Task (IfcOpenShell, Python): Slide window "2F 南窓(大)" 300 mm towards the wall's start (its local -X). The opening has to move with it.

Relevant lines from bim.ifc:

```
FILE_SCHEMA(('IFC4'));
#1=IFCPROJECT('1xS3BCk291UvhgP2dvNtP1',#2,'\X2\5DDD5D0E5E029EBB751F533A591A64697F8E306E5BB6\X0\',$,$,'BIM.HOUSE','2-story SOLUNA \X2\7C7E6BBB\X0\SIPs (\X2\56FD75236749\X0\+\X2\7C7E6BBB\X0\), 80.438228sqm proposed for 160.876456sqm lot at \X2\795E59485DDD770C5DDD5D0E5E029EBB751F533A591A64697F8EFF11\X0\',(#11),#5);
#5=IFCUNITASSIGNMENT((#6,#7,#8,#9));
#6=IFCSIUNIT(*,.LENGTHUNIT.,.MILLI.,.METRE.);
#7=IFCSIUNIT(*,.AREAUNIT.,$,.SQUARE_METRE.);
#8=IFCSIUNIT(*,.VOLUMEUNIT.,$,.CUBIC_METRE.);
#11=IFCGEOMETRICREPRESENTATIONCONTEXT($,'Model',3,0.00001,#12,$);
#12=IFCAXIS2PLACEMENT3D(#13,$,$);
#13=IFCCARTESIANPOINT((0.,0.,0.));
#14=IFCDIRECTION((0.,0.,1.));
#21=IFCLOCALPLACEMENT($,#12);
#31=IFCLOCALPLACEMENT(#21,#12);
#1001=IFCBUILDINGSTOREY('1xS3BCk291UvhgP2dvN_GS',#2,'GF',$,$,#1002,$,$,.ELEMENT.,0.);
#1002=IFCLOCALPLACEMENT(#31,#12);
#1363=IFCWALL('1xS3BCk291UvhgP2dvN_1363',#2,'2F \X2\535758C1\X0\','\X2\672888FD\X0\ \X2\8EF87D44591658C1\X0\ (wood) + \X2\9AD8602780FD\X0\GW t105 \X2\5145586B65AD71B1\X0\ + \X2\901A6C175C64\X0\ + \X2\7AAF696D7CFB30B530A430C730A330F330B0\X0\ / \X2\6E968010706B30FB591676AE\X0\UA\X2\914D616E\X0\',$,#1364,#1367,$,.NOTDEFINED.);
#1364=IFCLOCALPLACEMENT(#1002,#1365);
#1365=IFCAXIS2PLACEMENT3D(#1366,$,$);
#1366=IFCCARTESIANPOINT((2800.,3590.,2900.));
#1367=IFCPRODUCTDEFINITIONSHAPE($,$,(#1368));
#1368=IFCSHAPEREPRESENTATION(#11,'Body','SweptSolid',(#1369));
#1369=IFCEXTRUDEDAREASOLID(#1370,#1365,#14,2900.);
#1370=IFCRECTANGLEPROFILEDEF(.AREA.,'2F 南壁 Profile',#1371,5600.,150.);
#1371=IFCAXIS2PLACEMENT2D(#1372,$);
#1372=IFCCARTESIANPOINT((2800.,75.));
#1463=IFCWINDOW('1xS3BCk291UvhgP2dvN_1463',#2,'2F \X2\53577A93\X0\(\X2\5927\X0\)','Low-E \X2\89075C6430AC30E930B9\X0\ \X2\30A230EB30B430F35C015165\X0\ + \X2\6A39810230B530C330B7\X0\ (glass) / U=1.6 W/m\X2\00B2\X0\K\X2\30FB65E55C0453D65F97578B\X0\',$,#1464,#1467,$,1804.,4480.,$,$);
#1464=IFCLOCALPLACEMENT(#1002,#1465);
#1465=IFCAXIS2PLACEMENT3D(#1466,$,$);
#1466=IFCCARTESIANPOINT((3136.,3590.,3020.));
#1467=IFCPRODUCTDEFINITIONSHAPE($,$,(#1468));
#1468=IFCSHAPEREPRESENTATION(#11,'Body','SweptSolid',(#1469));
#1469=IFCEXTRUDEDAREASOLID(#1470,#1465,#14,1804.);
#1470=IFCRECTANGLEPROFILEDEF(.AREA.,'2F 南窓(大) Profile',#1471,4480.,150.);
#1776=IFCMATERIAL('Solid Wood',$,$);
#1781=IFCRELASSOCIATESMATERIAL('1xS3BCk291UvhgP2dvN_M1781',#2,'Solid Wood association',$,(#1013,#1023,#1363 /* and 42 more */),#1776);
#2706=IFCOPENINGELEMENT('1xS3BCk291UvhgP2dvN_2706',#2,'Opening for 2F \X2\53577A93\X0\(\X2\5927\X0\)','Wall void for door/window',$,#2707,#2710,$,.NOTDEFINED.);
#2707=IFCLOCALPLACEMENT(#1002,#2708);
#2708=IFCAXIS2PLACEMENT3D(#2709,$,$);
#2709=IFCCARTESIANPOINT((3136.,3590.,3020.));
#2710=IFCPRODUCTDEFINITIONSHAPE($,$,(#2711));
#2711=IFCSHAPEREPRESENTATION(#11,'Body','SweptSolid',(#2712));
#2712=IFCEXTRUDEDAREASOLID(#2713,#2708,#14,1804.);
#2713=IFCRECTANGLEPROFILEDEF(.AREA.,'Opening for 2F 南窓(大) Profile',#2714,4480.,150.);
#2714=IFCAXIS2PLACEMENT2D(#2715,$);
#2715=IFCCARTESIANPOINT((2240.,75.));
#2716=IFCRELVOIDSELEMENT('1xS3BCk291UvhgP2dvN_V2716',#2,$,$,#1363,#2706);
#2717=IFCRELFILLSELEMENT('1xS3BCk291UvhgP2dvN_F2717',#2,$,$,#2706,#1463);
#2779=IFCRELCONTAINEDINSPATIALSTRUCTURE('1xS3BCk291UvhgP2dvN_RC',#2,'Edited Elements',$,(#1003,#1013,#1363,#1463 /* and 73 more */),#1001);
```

```python
import ifcopenshell
import ifcopenshell.api.geometry
import ifcopenshell.util.placement

model = ifcopenshell.open("bim.ifc")

window = model.by_guid("1xS3BCk291UvhgP2dvN_1463")
opening = window.FillsVoids[0].RelatingOpeningElement
wall = opening.VoidsElements[0].RelatingBuildingElement

wall_matrix = ifcopenshell.util.placement.get_local_placement(wall.ObjectPlacement)
shift = wall_matrix[:3, 0] * -300.0
before = ifcopenshell.util.placement.get_local_placement(window.ObjectPlacement)[:3, 3].copy()

# The window is not placed relative to its opening, so move both.
for product in (opening, window):
    matrix = ifcopenshell.util.placement.get_local_placement(product.ObjectPlacement)
    matrix[:3, 3] += shift
    ifcopenshell.api.geometry.edit_object_placement(model, product=product, matrix=matrix, is_si=False)

after = ifcopenshell.util.placement.get_local_placement(window.ObjectPlacement)[:3, 3]
print("window moved by", (after - before).round(3) + 0.0)

model.write("bim_updated.ifc")
```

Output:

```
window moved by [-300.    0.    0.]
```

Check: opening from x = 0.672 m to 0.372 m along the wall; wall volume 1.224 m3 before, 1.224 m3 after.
